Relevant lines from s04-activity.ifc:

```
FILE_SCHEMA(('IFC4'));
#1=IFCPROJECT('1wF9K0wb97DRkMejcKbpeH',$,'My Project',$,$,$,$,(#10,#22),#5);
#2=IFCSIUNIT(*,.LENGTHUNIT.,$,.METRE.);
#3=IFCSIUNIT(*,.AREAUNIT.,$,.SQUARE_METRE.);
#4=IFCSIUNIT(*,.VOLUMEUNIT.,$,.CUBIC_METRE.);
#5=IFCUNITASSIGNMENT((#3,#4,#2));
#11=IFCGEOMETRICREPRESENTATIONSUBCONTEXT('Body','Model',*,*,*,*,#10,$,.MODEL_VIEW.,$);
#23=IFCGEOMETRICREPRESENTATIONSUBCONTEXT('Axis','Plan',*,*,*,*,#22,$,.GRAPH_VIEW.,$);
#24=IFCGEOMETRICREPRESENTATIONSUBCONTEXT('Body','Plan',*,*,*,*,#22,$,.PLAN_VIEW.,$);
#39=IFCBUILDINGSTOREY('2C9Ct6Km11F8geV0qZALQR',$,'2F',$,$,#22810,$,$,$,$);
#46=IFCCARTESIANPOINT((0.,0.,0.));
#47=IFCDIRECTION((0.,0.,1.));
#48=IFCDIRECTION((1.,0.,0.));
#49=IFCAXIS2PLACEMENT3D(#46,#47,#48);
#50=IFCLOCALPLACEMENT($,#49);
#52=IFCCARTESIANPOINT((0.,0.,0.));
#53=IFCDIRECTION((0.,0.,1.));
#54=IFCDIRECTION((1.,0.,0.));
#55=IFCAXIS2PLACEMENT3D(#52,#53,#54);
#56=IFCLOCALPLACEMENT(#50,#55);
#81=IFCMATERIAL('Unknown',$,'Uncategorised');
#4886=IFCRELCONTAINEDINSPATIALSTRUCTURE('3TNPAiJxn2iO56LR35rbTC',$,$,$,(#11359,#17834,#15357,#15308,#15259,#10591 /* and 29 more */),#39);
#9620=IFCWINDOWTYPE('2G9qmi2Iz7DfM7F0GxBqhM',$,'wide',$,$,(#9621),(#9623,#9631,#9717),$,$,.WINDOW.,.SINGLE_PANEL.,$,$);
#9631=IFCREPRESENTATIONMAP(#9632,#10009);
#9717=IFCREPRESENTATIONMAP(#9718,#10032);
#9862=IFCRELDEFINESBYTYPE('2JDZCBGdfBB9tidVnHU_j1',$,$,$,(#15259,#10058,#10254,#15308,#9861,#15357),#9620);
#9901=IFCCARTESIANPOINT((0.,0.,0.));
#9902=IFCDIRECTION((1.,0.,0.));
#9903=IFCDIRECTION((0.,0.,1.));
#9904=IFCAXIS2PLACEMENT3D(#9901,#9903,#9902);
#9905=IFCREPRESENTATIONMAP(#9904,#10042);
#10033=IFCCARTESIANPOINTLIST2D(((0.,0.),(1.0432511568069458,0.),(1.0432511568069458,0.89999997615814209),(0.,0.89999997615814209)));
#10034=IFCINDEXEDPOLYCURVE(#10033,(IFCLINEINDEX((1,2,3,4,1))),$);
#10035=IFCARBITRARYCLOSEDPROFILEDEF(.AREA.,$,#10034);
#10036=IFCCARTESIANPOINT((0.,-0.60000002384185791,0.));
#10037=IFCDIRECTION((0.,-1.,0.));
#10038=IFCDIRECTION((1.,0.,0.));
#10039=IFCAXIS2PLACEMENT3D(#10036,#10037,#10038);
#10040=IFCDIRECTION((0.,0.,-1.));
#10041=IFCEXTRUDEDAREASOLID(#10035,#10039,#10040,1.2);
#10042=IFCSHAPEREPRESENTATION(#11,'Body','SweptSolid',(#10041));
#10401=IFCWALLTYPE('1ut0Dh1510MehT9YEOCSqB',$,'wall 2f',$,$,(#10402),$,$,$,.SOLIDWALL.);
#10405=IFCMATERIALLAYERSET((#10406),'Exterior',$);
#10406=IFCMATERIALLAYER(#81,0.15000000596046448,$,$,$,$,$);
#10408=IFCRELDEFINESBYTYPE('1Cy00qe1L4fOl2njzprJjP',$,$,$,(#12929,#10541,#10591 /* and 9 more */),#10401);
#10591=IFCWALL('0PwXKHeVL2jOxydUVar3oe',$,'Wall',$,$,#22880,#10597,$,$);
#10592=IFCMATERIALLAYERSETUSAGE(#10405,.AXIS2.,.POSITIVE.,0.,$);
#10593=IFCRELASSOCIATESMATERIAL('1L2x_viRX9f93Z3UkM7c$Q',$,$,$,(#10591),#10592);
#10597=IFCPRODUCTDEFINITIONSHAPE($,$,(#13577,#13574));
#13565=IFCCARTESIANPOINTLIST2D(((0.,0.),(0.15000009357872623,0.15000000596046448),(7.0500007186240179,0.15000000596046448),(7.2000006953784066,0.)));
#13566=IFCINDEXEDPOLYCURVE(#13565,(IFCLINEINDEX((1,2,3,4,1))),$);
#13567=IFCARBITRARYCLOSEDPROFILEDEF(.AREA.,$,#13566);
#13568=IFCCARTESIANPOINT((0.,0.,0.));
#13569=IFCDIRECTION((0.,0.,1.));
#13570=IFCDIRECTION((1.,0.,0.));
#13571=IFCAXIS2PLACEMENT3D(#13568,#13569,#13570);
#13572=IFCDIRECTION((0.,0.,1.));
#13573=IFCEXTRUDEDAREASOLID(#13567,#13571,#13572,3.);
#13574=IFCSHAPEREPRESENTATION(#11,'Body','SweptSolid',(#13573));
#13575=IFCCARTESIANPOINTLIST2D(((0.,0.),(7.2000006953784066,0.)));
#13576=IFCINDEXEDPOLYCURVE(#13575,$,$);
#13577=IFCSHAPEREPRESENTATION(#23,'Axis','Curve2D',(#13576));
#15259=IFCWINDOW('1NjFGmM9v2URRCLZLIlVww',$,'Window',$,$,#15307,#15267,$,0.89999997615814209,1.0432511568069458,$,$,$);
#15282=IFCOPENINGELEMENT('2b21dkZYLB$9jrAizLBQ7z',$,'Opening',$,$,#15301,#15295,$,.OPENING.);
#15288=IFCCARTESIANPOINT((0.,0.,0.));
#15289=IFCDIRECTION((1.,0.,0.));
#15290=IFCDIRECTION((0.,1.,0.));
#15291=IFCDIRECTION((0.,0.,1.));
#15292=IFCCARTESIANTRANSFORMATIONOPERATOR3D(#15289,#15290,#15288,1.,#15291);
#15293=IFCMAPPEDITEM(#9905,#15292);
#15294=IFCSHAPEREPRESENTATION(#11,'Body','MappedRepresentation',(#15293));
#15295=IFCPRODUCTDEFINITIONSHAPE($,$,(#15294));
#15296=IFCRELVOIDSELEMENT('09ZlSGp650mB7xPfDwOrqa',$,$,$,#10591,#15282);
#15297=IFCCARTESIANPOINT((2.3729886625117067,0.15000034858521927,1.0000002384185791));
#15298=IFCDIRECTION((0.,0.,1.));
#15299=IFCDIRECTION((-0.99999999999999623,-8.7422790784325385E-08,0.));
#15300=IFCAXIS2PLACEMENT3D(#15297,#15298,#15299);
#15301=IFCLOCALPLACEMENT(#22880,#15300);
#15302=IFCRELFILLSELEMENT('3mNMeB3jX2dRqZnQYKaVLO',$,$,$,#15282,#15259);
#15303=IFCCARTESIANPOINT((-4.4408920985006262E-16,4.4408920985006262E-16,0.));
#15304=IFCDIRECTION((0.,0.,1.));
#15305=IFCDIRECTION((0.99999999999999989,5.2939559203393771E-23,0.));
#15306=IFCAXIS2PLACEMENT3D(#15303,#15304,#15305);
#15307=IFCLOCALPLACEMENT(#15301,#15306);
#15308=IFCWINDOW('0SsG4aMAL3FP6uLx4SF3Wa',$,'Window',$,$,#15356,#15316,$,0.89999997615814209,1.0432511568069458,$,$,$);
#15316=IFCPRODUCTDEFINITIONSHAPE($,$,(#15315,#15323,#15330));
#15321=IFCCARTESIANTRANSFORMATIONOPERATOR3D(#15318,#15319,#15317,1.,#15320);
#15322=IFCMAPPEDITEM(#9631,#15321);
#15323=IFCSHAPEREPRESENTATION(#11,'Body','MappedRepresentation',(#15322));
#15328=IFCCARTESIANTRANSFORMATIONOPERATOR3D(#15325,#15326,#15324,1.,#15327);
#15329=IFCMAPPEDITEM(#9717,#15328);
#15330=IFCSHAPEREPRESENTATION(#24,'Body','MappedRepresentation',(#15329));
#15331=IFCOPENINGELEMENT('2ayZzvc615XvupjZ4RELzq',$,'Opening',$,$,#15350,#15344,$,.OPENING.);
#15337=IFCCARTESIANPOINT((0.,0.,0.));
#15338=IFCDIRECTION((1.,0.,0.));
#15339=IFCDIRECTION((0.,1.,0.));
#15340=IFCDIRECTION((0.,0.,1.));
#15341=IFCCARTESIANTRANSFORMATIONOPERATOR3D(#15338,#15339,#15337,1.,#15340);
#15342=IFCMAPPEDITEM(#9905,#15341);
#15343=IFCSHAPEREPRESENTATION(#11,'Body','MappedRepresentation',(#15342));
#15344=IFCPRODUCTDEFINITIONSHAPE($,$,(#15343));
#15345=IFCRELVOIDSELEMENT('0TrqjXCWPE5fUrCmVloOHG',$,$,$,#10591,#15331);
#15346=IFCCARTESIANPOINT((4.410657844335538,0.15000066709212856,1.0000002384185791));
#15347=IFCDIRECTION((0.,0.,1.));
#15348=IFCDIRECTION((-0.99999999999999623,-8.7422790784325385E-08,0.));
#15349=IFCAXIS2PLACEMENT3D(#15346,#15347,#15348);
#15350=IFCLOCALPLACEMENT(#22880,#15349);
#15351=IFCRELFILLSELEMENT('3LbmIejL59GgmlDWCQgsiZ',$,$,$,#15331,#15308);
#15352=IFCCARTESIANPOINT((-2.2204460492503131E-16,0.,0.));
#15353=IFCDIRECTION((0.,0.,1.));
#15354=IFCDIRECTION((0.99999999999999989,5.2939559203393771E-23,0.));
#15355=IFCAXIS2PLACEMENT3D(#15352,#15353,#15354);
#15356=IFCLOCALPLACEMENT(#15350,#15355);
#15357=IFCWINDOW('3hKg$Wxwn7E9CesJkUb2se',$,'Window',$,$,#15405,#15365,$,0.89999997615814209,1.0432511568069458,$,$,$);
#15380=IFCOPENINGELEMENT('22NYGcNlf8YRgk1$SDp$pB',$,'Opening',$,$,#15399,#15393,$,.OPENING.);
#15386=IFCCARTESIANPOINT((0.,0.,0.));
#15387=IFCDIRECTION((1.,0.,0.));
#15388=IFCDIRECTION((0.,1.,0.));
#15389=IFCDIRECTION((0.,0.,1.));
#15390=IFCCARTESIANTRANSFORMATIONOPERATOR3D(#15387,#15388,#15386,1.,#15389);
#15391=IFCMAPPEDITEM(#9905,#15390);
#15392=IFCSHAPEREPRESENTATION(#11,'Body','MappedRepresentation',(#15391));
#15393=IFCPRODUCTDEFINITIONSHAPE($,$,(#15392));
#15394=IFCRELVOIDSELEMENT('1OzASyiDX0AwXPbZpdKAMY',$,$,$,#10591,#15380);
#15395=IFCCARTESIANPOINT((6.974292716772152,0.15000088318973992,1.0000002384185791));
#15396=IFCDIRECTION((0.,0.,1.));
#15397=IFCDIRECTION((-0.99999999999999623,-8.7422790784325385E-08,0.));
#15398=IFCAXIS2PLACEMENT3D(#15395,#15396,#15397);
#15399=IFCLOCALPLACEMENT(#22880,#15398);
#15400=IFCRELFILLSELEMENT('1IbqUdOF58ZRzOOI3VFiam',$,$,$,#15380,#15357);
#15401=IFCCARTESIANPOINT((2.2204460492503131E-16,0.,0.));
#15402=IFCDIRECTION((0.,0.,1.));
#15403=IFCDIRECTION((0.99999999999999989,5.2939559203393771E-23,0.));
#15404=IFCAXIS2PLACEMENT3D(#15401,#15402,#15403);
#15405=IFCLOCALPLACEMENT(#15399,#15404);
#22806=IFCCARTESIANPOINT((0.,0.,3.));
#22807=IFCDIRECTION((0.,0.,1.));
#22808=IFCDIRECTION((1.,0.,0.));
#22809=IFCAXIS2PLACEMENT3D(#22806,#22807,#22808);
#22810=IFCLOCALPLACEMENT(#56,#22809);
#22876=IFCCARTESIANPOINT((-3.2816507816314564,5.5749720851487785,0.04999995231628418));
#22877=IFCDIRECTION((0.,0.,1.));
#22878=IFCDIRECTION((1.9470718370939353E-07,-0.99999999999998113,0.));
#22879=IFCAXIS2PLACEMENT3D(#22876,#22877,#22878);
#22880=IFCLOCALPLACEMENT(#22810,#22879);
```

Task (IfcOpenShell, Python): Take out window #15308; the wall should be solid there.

```python
import ifcopenshell
import ifcopenshell.api.feature
import ifcopenshell.api.root
import ifcopenshell.geom
import ifcopenshell.util.shape

model = ifcopenshell.open("s04-activity.ifc")
settings = ifcopenshell.geom.settings()


def volume(element):
    """Net volume in cubic metres, openings subtracted."""
    shape = ifcopenshell.geom.create_shape(settings, element)
    return ifcopenshell.util.shape.get_volume(shape.geometry)


window = model.by_guid("0SsG4aMAL3FP6uLx4SF3Wa")
opening = window.FillsVoids[0].RelatingOpeningElement
wall = opening.VoidsElements[0].RelatingBuildingElement
before = volume(wall)

ifcopenshell.api.root.remove_product(model, product=window)
ifcopenshell.api.feature.remove_feature(model, feature=opening)

after = volume(wall)

print(f"wall volume {before:.3f} -> {after:.3f} m3")

model.write("s04-activity_edited.ifc")
```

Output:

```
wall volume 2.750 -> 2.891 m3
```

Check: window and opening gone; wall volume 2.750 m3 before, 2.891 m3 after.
